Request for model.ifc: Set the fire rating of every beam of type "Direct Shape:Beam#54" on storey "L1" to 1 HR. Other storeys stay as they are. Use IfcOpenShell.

First a look at what the model holds.

```python
import ifcopenshell
import ifcopenshell.util.element

model = ifcopenshell.open("model.ifc")
print(model.schema)
storey = next(s for s in model.by_type("IfcBuildingStorey") if s.Name == "L1")
beams = [e for e in ifcopenshell.util.element.get_decomposition(storey) if e.is_a("IfcBeam")]
seen = {}
for e in beams:
    element_type = ifcopenshell.util.element.get_type(e)
    key = (element_type.Name if element_type != e and element_type else None, ifcopenshell.util.element.get_pset(e, "Pset_BeamCommon", "FireRating"))
    seen[key] = seen.get(key, 0) + 1
for (name, value), count in sorted(seen.items(), key=str):
    print(count, "x", name, "|", value)
```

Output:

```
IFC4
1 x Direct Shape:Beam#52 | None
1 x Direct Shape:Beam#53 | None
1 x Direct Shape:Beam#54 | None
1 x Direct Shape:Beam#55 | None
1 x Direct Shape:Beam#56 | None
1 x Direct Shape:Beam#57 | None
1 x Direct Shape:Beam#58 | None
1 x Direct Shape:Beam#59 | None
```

```python
import ifcopenshell
import ifcopenshell.api.pset
import ifcopenshell.util.element

model = ifcopenshell.open("model.ifc")

storey = next(s for s in model.by_type("IfcBuildingStorey") if s.Name == "L1")
beams = [e for e in ifcopenshell.util.element.get_decomposition(storey) if e.is_a("IfcBeam")]

count = 0
for e in beams:
    element_type = ifcopenshell.util.element.get_type(e)
    if element_type in (None, e) or element_type.Name != "Direct Shape:Beam#54":
        continue
    # add_pset returns the element's existing set when there is one.
    pset = ifcopenshell.api.pset.add_pset(model, product=e, name="Pset_BeamCommon")
    ifcopenshell.api.pset.edit_pset(model, pset=pset, properties={"FireRating": "1 HR"})
    count += 1

print(count, "beams updated")

model.write("model_edited.ifc")
```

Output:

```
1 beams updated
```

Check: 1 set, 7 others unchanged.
